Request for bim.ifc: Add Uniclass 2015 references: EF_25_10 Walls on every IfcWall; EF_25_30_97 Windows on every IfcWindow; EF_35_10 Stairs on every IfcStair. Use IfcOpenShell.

First a look at what the model holds.

```python
import ifcopenshell

model = ifcopenshell.open("bim.ifc")
print(model.schema)
print("classifications:", [c.Name for c in model.by_type("IfcClassification")])
for ifc_class in ("IfcDoor", "IfcRoof", "IfcStair", "IfcWall", "IfcWindow"):
    print(ifc_class, len(model.by_type(ifc_class)))
```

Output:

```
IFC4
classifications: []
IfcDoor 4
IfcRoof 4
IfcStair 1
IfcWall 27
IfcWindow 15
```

```python
import ifcopenshell
import ifcopenshell.api.classification

model = ifcopenshell.open("bim.ifc")

system = ifcopenshell.api.classification.add_classification(model, classification="Uniclass 2015")

codes = {
    "IfcWall": ("EF_25_10", "Walls"),
    "IfcWindow": ("EF_25_30_97", "Windows"),
    "IfcStair": ("EF_35_10", "Stairs"),
}
for ifc_class, (code, name) in codes.items():
    products = model.by_type(ifc_class)
    ifcopenshell.api.classification.add_reference(
        model, products=products, classification=system, identification=code, name=name
    )
    print(code, len(products))

model.write("bim_edited.ifc")
```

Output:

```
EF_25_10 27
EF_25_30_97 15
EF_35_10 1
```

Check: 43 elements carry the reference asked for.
